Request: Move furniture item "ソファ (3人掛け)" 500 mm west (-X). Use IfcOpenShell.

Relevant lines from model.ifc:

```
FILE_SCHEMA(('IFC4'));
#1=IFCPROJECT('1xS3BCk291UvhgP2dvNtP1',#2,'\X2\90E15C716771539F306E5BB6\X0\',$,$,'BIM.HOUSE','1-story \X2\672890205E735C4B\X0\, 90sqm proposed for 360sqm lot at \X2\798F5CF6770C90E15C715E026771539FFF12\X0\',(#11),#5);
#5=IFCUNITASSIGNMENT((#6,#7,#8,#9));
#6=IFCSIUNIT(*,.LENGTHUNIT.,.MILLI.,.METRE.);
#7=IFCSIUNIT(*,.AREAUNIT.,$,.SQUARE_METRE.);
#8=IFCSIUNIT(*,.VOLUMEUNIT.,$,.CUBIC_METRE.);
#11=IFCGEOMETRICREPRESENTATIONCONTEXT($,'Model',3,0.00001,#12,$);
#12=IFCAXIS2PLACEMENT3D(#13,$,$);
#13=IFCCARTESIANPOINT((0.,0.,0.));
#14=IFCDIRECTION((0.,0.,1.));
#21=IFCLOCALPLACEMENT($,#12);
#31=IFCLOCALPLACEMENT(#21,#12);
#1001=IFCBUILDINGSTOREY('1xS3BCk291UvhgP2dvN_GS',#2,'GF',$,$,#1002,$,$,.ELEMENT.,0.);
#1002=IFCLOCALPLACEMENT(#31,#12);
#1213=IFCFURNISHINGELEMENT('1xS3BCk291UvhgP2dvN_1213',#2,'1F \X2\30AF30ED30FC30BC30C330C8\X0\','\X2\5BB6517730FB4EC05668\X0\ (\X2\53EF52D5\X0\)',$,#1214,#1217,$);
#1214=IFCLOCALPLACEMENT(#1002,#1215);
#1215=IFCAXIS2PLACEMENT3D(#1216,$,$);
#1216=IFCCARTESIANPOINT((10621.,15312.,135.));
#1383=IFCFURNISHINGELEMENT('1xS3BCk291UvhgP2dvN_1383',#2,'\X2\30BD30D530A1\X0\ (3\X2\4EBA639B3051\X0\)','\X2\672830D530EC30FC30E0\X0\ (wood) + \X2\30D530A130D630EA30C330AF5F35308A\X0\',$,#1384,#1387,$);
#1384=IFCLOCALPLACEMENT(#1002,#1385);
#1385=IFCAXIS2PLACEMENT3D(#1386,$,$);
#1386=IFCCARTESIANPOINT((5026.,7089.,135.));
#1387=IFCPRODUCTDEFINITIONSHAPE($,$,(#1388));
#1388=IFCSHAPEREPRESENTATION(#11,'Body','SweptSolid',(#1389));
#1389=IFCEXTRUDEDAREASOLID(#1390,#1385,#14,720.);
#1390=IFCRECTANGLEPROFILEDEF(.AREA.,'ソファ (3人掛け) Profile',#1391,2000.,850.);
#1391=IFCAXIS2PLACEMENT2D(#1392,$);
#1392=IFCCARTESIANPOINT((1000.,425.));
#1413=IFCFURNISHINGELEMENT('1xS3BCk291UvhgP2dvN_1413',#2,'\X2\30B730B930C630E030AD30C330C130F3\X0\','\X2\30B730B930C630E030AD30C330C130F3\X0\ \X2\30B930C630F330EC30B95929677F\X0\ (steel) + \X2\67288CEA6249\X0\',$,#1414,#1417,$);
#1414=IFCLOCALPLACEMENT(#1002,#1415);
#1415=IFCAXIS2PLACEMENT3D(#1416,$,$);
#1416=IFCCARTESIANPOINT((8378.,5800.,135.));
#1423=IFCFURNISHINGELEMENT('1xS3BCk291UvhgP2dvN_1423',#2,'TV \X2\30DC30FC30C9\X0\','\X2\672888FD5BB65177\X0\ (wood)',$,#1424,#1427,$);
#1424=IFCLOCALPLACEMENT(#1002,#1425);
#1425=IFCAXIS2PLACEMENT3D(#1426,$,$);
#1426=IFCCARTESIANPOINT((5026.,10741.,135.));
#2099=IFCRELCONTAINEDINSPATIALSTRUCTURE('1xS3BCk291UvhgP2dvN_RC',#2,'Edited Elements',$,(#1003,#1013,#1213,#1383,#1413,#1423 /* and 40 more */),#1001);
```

```python
import ifcopenshell
import ifcopenshell.api.geometry
import ifcopenshell.util.placement

model = ifcopenshell.open("model.ifc")

item = model.by_guid("1xS3BCk291UvhgP2dvN_1383")
matrix = ifcopenshell.util.placement.get_local_placement(item.ObjectPlacement)
matrix[0, 3] -= 500.0
ifcopenshell.api.geometry.edit_object_placement(model, product=item, matrix=matrix, is_si=False)

print(ifcopenshell.util.placement.get_local_placement(item.ObjectPlacement).round(3) + 0.0)

model.write("model_v2.ifc")
```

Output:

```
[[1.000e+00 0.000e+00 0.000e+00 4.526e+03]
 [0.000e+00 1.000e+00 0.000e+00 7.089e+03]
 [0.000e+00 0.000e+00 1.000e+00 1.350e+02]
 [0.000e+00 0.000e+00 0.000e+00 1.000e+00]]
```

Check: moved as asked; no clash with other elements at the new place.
